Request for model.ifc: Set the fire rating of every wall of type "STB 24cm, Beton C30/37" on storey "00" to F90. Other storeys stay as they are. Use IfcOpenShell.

First a look at what the model holds.

```python
import ifcopenshell
import ifcopenshell.util.element

model = ifcopenshell.open("model.ifc")
print(model.schema)
storey = next(s for s in model.by_type("IfcBuildingStorey") if s.Name == "00")
walls = [e for e in ifcopenshell.util.element.get_decomposition(storey) if e.is_a("IfcWall")]
seen = {}
for e in walls:
    element_type = ifcopenshell.util.element.get_type(e)
    key = (element_type.Name if element_type != e and element_type else None, ifcopenshell.util.element.get_pset(e, "Pset_WallCommon", "FireRating"))
    seen[key] = seen.get(key, 0) + 1
for (name, value), count in sorted(seen.items(), key=str):
    print(count, "x", name, "|", value)
```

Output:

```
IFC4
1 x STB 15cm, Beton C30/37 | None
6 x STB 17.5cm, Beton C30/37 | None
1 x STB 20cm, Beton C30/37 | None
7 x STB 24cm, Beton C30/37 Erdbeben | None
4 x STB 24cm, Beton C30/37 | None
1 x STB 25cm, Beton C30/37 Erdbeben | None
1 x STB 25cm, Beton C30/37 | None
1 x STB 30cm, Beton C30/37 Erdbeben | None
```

```python
import ifcopenshell
import ifcopenshell.api.pset
import ifcopenshell.util.element

model = ifcopenshell.open("model.ifc")

storey = next(s for s in model.by_type("IfcBuildingStorey") if s.Name == "00")
walls = [e for e in ifcopenshell.util.element.get_decomposition(storey) if e.is_a("IfcWall")]

count = 0
for e in walls:
    element_type = ifcopenshell.util.element.get_type(e)
    if element_type in (None, e) or element_type.Name != "STB 24cm, Beton C30/37":
        continue
    # add_pset returns the element's existing set when there is one.
    pset = ifcopenshell.api.pset.add_pset(model, product=e, name="Pset_WallCommon")
    ifcopenshell.api.pset.edit_pset(model, pset=pset, properties={"FireRating": "F90"})
    count += 1

print(count, "walls updated")

model.write("model_rev.ifc")
```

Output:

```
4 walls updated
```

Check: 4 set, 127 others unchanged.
